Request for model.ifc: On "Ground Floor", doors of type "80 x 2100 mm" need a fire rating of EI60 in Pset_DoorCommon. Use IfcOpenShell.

First a look at what the model holds.

```python
import ifcopenshell
import ifcopenshell.util.element

model = ifcopenshell.open("model.ifc")
print(model.schema)
storey = next(s for s in model.by_type("IfcBuildingStorey") if s.Name == "Ground Floor")
doors = [e for e in ifcopenshell.util.element.get_decomposition(storey) if e.is_a("IfcDoor")]
seen = {}
for e in doors:
    element_type = ifcopenshell.util.element.get_type(e)
    key = (element_type.Name if element_type != e and element_type else None, ifcopenshell.util.element.get_pset(e, "Pset_DoorCommon", "FireRating"))
    seen[key] = seen.get(key, 0) + 1
for (name, value), count in sorted(seen.items(), key=str):
    print(count, "x", name, "|", value)
```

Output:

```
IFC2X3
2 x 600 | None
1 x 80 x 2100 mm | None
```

```python
import ifcopenshell
import ifcopenshell.api.pset
import ifcopenshell.util.element

model = ifcopenshell.open("model.ifc")

storey = next(s for s in model.by_type("IfcBuildingStorey") if s.Name == "Ground Floor")
doors = [e for e in ifcopenshell.util.element.get_decomposition(storey) if e.is_a("IfcDoor")]

count = 0
for e in doors:
    element_type = ifcopenshell.util.element.get_type(e)
    if element_type in (None, e) or element_type.Name != "80 x 2100 mm":
        continue
    # add_pset returns the element's existing set when there is one.
    pset = ifcopenshell.api.pset.add_pset(model, product=e, name="Pset_DoorCommon")
    ifcopenshell.api.pset.edit_pset(model, pset=pset, properties={"FireRating": "EI60"})
    count += 1

print(count, "doors updated")

model.write("model_rev.ifc")
```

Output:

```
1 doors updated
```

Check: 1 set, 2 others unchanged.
